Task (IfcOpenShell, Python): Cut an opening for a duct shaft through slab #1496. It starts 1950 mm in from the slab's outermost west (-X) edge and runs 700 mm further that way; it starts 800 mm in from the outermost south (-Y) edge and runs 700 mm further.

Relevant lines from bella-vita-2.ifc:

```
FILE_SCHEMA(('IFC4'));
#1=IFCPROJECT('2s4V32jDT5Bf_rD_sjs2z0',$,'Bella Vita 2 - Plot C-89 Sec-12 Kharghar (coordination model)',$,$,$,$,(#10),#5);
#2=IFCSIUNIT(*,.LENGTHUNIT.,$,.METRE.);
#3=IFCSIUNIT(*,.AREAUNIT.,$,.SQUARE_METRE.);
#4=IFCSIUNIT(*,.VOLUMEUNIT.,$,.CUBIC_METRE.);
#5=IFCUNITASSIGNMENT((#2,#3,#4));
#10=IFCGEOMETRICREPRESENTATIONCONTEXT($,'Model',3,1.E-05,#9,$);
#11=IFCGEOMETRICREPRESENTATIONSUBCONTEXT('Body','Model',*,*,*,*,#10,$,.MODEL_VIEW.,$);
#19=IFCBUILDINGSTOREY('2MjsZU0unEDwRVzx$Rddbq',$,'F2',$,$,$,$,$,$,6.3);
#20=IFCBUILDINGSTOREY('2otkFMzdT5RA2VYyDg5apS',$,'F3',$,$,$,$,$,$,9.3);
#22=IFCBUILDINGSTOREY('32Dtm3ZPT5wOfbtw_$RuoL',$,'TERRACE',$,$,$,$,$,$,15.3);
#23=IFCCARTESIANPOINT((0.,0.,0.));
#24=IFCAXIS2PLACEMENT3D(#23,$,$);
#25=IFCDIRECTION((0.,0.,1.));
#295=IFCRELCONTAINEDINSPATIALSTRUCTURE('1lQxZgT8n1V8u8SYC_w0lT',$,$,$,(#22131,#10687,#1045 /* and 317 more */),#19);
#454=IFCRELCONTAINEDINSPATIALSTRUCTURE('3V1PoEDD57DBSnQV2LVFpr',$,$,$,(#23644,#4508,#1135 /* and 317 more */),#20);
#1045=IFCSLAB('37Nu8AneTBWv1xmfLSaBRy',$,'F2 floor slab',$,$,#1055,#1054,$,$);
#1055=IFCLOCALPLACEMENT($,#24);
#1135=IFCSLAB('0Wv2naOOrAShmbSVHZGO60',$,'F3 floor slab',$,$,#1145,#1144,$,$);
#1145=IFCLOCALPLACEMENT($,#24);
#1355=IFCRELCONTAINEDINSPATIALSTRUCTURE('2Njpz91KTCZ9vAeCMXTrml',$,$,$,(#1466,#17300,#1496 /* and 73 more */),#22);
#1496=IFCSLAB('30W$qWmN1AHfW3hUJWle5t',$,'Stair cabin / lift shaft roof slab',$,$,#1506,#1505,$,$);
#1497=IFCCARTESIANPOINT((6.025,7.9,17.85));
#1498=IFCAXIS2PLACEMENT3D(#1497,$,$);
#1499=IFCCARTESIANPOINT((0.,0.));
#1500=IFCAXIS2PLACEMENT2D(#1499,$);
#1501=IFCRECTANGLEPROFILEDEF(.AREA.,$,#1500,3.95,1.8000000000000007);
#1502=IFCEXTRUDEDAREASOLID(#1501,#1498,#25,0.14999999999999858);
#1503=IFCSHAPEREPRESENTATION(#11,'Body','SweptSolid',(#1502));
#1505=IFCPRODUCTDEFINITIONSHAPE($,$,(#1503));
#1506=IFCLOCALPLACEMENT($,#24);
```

```python
import numpy as np
import ifcopenshell
import ifcopenshell.api.feature
import ifcopenshell.api.geometry
import ifcopenshell.api.root
import ifcopenshell.geom
import ifcopenshell.util.placement
import ifcopenshell.util.representation
import ifcopenshell.util.shape
import ifcopenshell.util.unit

model = ifcopenshell.open("bella-vita-2.ifc")
unit_scale = ifcopenshell.util.unit.calculate_unit_scale(model)
settings = ifcopenshell.geom.settings()


def volume(element):
    """Net volume in cubic metres, openings subtracted."""
    shape = ifcopenshell.geom.create_shape(settings, element)
    return ifcopenshell.util.shape.get_volume(shape.geometry)


slab = model.by_guid("30W$qWmN1AHfW3hUJWle5t")
before = volume(slab)

# Extent in the slab's own axes, in metres. The edges named are its -X and -Y sides.
slab_shape = ifcopenshell.geom.create_shape(settings, slab)
vertices = ifcopenshell.util.shape.get_vertices(slab_shape.geometry)
x_min, y_min, bottom = vertices.min(axis=0)
top = vertices[:, 2].max()

opening = ifcopenshell.api.root.create_entity(model, ifc_class="IfcOpeningElement", name="Duct shaft opening", predefined_type="OPENING")
context = ifcopenshell.util.representation.get_context(model, "Model", "Body", "MODEL_VIEW")
width, depth = 0.7, 0.7
outline = [(0.0, 0.0), (width, 0.0), (width, depth), (0.0, depth), (0.0, 0.0)]
# Overshoot both faces by 50 mm so the cut is clean.
shape = ifcopenshell.api.geometry.add_slab_representation(
    model, context=context, depth=top - bottom + 0.1, polyline=outline
)
ifcopenshell.api.geometry.assign_representation(model, product=opening, representation=shape)

matrix = ifcopenshell.util.placement.get_local_placement(slab.ObjectPlacement)
matrix[:, 3] = matrix @ np.append(np.array([x_min + 1.95, y_min + 0.8, bottom - 0.05]) / unit_scale, 1.0)
ifcopenshell.api.geometry.edit_object_placement(model, product=opening, matrix=matrix, is_si=False)
ifcopenshell.api.feature.add_feature(model, feature=opening, element=slab)

after = volume(slab)

print(f"slab volume {before:.3f} -> {after:.3f} m3")

model.write("bella-vita-2-out.ifc")
```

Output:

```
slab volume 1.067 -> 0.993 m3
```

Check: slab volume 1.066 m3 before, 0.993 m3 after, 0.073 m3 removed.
